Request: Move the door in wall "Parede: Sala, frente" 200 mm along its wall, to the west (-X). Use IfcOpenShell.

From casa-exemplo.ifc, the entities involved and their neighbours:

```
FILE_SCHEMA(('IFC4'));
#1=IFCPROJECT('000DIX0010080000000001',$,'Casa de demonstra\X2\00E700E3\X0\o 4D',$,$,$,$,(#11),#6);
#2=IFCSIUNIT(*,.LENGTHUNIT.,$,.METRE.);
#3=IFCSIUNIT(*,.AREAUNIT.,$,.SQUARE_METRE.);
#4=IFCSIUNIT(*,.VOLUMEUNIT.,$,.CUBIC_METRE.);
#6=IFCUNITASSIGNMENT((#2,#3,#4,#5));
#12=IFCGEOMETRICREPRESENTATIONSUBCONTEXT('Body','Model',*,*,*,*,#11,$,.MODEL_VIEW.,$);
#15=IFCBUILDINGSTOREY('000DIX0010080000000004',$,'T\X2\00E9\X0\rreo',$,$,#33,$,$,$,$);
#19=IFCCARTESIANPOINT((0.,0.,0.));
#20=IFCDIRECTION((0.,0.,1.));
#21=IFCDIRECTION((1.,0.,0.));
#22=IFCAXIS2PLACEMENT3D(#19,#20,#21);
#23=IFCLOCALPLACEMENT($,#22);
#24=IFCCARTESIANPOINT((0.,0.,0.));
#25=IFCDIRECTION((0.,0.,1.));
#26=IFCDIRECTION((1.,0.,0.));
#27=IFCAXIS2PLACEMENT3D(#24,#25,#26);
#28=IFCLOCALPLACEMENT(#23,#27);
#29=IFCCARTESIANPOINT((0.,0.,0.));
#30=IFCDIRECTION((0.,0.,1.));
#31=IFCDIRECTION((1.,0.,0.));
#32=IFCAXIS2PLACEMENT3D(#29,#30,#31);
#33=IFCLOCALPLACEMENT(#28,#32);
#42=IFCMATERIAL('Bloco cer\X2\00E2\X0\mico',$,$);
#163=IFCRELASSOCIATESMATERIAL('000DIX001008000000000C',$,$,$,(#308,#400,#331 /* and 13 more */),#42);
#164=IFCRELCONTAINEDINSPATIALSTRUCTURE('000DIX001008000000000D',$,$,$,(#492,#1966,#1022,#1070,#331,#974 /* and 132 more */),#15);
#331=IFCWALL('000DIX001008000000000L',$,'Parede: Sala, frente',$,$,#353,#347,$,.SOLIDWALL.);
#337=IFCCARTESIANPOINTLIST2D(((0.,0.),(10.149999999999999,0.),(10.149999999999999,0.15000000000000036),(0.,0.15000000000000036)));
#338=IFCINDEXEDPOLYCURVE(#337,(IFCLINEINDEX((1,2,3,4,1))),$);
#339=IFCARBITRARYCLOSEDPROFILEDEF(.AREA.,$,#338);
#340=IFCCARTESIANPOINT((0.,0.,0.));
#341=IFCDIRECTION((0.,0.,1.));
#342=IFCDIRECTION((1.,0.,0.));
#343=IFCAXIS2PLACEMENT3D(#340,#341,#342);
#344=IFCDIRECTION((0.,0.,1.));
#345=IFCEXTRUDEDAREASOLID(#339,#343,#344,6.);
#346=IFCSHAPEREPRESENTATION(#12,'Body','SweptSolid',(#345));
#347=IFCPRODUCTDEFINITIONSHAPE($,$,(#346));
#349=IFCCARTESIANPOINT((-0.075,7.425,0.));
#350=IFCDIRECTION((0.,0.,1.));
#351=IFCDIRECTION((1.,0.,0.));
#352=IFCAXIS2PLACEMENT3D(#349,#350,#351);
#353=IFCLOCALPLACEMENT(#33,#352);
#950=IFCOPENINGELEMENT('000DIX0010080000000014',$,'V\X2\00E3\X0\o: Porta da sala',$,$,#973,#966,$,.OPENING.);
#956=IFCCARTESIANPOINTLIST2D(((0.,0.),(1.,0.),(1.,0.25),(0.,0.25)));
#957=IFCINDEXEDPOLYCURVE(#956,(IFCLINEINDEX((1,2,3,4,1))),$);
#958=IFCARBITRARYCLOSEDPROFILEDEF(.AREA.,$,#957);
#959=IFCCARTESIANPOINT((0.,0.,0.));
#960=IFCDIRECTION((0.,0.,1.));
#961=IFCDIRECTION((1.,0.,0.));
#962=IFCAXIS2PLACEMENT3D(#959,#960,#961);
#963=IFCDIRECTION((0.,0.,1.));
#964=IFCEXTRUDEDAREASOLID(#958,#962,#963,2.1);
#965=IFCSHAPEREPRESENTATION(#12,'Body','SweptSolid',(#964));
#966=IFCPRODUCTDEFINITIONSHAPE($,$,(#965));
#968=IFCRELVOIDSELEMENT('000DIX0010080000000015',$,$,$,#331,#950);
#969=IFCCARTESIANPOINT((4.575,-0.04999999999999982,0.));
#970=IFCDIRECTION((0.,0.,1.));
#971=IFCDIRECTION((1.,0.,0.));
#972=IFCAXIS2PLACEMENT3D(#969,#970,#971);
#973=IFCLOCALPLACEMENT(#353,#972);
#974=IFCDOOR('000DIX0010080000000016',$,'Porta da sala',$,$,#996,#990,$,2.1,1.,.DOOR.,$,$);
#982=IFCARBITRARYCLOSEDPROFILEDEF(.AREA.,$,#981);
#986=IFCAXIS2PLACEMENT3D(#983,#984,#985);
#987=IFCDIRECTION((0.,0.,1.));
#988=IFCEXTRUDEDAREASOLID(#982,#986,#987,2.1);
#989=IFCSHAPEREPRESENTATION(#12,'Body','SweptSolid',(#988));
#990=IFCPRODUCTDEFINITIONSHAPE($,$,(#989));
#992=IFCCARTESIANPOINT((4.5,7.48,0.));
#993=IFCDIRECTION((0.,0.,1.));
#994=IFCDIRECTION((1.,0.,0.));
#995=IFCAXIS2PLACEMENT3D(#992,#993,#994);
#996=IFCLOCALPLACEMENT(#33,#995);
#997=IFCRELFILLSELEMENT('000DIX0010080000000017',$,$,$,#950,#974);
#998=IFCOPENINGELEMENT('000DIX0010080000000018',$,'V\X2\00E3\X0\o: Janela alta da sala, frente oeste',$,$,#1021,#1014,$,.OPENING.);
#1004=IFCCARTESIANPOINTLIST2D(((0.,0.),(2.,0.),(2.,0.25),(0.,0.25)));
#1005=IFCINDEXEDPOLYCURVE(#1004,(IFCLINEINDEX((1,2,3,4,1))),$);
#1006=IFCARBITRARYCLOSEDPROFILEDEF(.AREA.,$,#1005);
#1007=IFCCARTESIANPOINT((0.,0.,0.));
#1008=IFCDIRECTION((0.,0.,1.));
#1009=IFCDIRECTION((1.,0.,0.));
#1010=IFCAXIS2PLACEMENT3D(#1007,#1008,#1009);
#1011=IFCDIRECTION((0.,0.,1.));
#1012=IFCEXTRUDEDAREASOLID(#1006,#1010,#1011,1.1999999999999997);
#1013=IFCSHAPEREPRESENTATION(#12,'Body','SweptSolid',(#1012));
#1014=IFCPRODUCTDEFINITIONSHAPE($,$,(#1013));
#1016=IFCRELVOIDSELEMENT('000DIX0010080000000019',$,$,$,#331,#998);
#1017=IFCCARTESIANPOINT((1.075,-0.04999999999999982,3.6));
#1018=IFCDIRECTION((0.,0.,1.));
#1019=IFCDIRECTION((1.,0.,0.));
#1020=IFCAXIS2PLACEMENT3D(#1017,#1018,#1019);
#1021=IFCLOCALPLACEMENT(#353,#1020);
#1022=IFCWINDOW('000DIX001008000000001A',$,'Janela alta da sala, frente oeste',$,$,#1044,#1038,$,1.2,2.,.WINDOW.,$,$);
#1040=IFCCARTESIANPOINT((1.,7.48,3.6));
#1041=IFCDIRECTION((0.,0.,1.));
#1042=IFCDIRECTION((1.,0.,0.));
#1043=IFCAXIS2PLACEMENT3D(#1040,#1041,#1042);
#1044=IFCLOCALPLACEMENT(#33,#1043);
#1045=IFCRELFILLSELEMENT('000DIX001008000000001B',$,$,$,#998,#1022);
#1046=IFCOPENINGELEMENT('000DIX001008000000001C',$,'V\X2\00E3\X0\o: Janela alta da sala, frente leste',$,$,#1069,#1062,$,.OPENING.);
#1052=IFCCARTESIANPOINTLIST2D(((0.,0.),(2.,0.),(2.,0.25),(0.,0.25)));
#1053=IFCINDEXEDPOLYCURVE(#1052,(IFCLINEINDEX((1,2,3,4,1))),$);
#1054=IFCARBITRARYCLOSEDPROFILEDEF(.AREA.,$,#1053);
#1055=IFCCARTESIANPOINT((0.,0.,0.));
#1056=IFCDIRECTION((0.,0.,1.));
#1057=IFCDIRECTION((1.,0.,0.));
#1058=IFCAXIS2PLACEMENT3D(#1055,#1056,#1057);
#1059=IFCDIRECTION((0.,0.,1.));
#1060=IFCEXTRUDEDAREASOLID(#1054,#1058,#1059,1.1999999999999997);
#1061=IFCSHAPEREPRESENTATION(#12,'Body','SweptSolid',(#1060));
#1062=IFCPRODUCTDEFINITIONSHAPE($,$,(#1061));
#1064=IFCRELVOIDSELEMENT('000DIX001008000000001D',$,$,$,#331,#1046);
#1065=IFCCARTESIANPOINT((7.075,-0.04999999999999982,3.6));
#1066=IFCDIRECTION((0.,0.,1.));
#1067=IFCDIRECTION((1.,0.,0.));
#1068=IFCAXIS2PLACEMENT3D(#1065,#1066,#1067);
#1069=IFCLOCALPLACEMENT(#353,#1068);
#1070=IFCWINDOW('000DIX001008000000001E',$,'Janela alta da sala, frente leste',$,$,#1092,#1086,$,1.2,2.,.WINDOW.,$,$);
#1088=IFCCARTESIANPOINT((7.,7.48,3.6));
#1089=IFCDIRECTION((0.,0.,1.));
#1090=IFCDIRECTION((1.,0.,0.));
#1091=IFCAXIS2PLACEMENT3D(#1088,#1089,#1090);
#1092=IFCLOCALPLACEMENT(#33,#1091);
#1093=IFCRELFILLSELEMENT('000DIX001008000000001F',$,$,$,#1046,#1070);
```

```python
import ifcopenshell
import ifcopenshell.api.geometry
import ifcopenshell.util.placement
import ifcopenshell.util.unit

model = ifcopenshell.open("casa-exemplo.ifc")
unit_scale = ifcopenshell.util.unit.calculate_unit_scale(model)

door = model.by_guid("000DIX0010080000000016")
opening = door.FillsVoids[0].RelatingOpeningElement
wall = opening.VoidsElements[0].RelatingBuildingElement

wall_matrix = ifcopenshell.util.placement.get_local_placement(wall.ObjectPlacement)
shift = wall_matrix[:3, 0] * -0.2 / unit_scale
before = ifcopenshell.util.placement.get_local_placement(door.ObjectPlacement)[:3, 3].copy()

# The door is not placed relative to its opening, so move both.
for product in (opening, door):
    matrix = ifcopenshell.util.placement.get_local_placement(product.ObjectPlacement)
    matrix[:3, 3] += shift
    ifcopenshell.api.geometry.edit_object_placement(model, product=product, matrix=matrix, is_si=False)

after = ifcopenshell.util.placement.get_local_placement(door.ObjectPlacement)[:3, 3]
print("door moved by", (after - before).round(3) + 0.0)

model.write("casa-exemplo_edited.ifc")
```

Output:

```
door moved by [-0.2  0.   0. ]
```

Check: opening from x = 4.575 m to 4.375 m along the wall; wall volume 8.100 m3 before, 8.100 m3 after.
